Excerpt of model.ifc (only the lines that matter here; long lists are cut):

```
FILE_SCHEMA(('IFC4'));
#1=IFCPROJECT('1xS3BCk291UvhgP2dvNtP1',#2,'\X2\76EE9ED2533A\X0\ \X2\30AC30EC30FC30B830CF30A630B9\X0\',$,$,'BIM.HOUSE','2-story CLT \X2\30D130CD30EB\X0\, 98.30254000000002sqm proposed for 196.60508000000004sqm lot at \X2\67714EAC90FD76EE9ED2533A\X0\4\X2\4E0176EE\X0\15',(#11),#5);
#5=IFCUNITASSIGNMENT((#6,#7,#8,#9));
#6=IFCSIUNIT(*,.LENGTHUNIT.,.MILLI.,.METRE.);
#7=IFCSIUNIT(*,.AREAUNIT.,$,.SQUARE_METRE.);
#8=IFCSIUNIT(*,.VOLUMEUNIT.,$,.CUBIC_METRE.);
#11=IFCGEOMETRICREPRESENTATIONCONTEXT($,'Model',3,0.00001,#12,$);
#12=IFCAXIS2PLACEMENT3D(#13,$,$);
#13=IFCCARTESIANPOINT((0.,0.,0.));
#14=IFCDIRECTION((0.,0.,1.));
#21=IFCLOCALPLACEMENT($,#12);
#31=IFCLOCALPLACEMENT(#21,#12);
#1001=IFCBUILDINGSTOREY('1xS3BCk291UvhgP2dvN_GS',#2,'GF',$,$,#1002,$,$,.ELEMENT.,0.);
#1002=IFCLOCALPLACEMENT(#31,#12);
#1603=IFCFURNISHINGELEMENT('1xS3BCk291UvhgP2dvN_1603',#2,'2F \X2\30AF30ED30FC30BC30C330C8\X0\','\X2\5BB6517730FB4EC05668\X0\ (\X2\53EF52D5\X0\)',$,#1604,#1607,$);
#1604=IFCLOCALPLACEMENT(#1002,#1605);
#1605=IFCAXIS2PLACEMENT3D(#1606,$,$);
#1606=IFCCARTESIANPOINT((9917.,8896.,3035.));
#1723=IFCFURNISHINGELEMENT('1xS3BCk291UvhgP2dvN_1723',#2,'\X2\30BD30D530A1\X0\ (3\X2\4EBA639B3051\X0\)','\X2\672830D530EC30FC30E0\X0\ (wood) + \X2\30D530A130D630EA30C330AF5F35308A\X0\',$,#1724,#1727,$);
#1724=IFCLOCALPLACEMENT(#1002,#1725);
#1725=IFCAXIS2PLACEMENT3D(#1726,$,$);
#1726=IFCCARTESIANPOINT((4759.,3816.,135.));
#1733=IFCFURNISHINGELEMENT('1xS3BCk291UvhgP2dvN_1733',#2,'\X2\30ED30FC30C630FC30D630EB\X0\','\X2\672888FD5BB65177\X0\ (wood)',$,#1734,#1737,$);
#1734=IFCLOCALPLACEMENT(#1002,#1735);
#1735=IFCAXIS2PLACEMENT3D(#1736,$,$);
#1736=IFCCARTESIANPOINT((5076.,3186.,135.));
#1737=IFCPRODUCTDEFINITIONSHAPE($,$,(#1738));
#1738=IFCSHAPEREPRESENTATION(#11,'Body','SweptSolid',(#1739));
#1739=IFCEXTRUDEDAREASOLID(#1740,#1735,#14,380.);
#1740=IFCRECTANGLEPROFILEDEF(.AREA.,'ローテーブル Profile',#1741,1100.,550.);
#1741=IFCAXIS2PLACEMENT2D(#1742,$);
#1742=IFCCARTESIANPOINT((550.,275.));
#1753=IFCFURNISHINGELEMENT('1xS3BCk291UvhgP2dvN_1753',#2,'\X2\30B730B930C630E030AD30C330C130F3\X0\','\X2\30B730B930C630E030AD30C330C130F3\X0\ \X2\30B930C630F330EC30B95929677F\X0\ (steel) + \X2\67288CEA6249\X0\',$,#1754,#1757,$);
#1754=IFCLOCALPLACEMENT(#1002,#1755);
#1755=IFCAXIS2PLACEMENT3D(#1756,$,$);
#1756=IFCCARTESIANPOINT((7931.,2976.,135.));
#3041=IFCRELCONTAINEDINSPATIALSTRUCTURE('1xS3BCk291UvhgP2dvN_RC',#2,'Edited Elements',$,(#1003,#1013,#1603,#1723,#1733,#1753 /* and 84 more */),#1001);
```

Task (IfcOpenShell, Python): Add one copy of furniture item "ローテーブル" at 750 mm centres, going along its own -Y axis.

```python
import ifcopenshell
import ifcopenshell.api.geometry
import ifcopenshell.api.root
import ifcopenshell.util.element
import ifcopenshell.util.placement
import ifcopenshell.util.unit

model = ifcopenshell.open("model.ifc")
unit_scale = ifcopenshell.util.unit.calculate_unit_scale(model)


def reuse_history(source, copy):
    """copy_class also copies each property set's owner history, people and application; keep the originals."""
    for rel in copy.IsDefinedBy:
        if rel.is_a("IfcRelDefinesByProperties") and (history := rel.RelatingPropertyDefinition.OwnerHistory):
            rel.RelatingPropertyDefinition.OwnerHistory = source.OwnerHistory
            ifcopenshell.util.element.remove_deep2(model, history)


source = model.by_guid("1xS3BCk291UvhgP2dvN_1733")
base = ifcopenshell.util.placement.get_local_placement(source.ObjectPlacement)
step = -base[:3, 1] * 0.75 / unit_scale

for i in range(1, 2):
    copy = ifcopenshell.api.root.copy_class(model, product=source)
    copy.Representation = ifcopenshell.util.element.copy_deep(
        model, source.Representation, exclude=["IfcGeometricRepresentationContext", "IfcRepresentationMap"]
    )
    reuse_history(source, copy)
    matrix = base.copy()
    matrix[:3, 3] += i * step
    print("added at", matrix[:3, 3].round(3) + 0.0)
    ifcopenshell.api.geometry.edit_object_placement(model, product=copy, matrix=matrix, is_si=False)

model.write("model-out.ifc")
```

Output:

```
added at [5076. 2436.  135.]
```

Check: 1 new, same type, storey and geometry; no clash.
